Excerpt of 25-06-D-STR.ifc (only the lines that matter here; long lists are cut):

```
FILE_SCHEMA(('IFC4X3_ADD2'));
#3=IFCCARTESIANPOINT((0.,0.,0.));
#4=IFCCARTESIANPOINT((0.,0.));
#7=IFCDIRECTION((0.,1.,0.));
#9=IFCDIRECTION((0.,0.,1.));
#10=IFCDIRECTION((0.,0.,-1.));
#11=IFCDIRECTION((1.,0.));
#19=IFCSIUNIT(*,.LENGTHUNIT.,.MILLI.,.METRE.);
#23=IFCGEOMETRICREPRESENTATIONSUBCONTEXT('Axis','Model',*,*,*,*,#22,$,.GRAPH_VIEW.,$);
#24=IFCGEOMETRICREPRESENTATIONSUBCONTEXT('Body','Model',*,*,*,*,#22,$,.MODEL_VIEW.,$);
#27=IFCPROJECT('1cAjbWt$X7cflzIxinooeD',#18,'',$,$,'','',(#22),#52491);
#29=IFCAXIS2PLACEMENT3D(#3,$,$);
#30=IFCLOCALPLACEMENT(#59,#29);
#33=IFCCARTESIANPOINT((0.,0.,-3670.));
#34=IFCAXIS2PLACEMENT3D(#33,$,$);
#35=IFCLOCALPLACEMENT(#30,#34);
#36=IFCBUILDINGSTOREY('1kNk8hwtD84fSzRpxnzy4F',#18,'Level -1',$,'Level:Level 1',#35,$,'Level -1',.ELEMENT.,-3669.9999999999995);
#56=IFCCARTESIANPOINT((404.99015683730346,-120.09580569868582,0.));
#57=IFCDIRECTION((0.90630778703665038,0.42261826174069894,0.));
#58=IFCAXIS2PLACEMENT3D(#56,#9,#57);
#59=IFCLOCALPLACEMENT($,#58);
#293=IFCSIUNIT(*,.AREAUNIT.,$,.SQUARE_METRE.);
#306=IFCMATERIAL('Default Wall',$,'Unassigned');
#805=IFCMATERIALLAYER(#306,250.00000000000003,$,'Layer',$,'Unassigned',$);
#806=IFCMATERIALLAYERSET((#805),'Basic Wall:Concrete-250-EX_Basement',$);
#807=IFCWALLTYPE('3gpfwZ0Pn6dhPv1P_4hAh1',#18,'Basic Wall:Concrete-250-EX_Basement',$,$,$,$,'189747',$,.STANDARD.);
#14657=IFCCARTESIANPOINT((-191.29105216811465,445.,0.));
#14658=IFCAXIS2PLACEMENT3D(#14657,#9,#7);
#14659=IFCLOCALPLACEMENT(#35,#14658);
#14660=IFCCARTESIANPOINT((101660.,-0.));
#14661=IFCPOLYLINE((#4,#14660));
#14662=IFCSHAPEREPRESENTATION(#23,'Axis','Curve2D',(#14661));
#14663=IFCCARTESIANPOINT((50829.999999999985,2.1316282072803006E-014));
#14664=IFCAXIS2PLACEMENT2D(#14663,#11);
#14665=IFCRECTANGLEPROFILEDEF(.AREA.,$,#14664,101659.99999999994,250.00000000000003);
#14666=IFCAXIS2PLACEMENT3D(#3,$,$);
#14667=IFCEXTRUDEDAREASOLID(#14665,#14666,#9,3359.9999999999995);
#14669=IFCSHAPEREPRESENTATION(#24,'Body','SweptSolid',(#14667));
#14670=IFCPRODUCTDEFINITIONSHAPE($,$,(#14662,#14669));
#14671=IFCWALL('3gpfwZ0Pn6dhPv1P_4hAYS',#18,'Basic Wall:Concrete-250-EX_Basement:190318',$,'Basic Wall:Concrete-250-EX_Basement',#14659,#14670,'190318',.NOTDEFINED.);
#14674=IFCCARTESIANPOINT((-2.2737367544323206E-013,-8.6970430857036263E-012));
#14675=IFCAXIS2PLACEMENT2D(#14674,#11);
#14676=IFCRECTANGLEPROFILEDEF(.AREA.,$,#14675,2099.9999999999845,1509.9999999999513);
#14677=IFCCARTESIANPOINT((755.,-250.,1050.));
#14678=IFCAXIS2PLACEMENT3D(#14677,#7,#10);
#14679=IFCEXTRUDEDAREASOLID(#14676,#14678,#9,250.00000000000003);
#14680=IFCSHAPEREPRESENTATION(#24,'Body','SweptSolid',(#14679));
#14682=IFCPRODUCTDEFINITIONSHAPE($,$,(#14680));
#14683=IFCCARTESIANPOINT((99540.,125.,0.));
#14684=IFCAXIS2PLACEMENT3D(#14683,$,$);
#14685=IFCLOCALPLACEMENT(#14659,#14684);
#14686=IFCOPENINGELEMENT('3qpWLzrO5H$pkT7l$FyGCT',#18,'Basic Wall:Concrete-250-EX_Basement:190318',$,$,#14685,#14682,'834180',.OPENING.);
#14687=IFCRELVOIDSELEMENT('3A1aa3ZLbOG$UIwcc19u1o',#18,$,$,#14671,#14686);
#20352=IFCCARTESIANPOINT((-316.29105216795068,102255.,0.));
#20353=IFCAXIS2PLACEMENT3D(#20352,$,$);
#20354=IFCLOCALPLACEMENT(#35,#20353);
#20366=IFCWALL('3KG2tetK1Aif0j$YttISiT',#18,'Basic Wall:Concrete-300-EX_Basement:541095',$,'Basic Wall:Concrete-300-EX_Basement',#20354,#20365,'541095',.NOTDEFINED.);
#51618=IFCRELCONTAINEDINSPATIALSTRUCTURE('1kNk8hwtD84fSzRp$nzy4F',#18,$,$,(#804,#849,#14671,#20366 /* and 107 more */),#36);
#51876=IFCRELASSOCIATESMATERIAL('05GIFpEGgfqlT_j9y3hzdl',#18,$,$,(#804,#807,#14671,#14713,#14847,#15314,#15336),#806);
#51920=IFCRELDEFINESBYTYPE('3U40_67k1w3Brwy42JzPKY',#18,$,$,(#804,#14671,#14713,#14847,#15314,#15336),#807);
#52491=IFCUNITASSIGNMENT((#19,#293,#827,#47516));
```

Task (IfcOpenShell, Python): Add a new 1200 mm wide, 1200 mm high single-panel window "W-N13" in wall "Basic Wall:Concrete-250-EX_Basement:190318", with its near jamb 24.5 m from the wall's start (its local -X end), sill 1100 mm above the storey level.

```python
import numpy as np
import ifcopenshell
import ifcopenshell.api.feature
import ifcopenshell.api.geometry
import ifcopenshell.api.root
import ifcopenshell.api.spatial
import ifcopenshell.geom
import ifcopenshell.util.element
import ifcopenshell.util.placement
import ifcopenshell.util.representation
import ifcopenshell.util.shape
import ifcopenshell.util.unit

model = ifcopenshell.open("25-06-D-STR.ifc")
unit_scale = ifcopenshell.util.unit.calculate_unit_scale(model)
settings = ifcopenshell.geom.settings()


def volume(element):
    """Net volume in cubic metres, openings subtracted."""
    shape = ifcopenshell.geom.create_shape(settings, element)
    return ifcopenshell.util.shape.get_volume(shape.geometry)


wall = model.by_guid("3gpfwZ0Pn6dhPv1P_4hAYS")
storey = ifcopenshell.util.element.get_container(wall, ifc_class="IfcBuildingStorey")
context = ifcopenshell.util.representation.get_context(model, "Model", "Body", "MODEL_VIEW")
before = volume(wall)

width, height, from_end, sill = 1.2, 1.2, 24.5, 1.1  # metres

# The wall runs along its own X axis, and the end named is its -X end.
wall_shape = ifcopenshell.geom.create_shape(settings, wall)
x, y, z = ifcopenshell.util.shape.get_vertices(wall_shape.geometry).T
start = x.min() + from_end
face, thickness = float(y.min()), float(y.max() - y.min())
wall_matrix = ifcopenshell.util.placement.get_local_placement(wall.ObjectPlacement)
level = ifcopenshell.util.placement.get_local_placement(storey.ObjectPlacement)[2, 3]


def in_wall(x, y):
    """Placement at x, y metres in the wall's axes, at sill height."""
    matrix = wall_matrix.copy()
    matrix[:, 3] = wall_matrix @ np.array([x / unit_scale, y / unit_scale, 0.0, 1.0])
    matrix[2, 3] = level + sill / unit_scale
    return matrix


# Opening: a box that overshoots both wall faces by 50 mm.
opening = ifcopenshell.api.root.create_entity(model, ifc_class="IfcOpeningElement", predefined_type="OPENING")
box = ifcopenshell.api.geometry.add_wall_representation(
    model, context=context, length=width, height=height, thickness=thickness + 0.1
)
ifcopenshell.api.geometry.assign_representation(model, product=opening, representation=box)
ifcopenshell.api.geometry.edit_object_placement(model, product=opening, matrix=in_wall(start, face - 0.05), is_si=False)
ifcopenshell.api.feature.add_feature(model, feature=opening, element=wall)

window = ifcopenshell.api.root.create_entity(model, ifc_class="IfcWindow", name="W-N13", predefined_type="WINDOW")
window.OverallWidth, window.OverallHeight = width / unit_scale, height / unit_scale
window.PartitioningType = "SINGLE_PANEL"
body = ifcopenshell.api.geometry.add_window_representation(
    model,
    context=context,
    overall_width=window.OverallWidth,
    overall_height=window.OverallHeight,
    partition_type="SINGLE_PANEL",
)
ifcopenshell.api.geometry.assign_representation(model, product=window, representation=body)
ifcopenshell.api.spatial.assign_container(model, products=[window], relating_structure=storey)
ifcopenshell.api.feature.add_filling(model, opening=opening, element=window)

# Centre the window in the wall's thickness.
ifcopenshell.api.geometry.edit_object_placement(model, product=window, matrix=in_wall(start, face), is_si=False)
window_shape = ifcopenshell.geom.create_shape(settings, window)
depth = ifcopenshell.util.shape.get_vertices(window_shape.geometry)[:, 1]
offset = face + thickness / 2 - (depth.min() + depth.max()) / 2
ifcopenshell.api.geometry.edit_object_placement(model, product=window, matrix=in_wall(start, offset), is_si=False)

after = volume(wall)

print(f"wall volume {before:.3f} -> {after:.3f} m3")

model.write("25-06-D-STR-out.ifc")
```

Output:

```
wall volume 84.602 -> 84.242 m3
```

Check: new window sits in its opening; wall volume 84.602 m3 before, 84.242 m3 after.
